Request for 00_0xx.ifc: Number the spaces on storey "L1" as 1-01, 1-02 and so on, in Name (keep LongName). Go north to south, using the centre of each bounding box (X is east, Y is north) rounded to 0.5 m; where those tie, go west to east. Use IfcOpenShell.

First a look at what the model holds.

```python
import ifcopenshell
import ifcopenshell.util.element
import ifcopenshell.util.placement

model = ifcopenshell.open("00_0xx.ifc")
print(model.schema)
storey = next(s for s in model.by_type("IfcBuildingStorey") if s.Name == "L1")
spaces = [e for e in ifcopenshell.util.element.get_decomposition(storey) if e.is_a("IfcSpace")]
for e in sorted(spaces, key=lambda e: e.id()):
    origin = ifcopenshell.util.placement.get_local_placement(e.ObjectPlacement)[:3, 3]
    print(e.id(), e.Name, e.LongName, origin.round(2) + 0.0, sep=" | ")
```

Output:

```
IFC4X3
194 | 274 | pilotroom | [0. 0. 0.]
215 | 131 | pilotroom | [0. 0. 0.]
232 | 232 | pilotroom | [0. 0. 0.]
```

```python
import ifcopenshell
import ifcopenshell.geom
import ifcopenshell.util.element
import ifcopenshell.util.shape

model = ifcopenshell.open("00_0xx.ifc")
settings = ifcopenshell.geom.settings()
settings.set("use-world-coords", True)


def centre(element):
    shape = ifcopenshell.geom.create_shape(settings, element)
    return ifcopenshell.util.shape.get_bbox_centroid(shape.geometry)


storey = next(s for s in model.by_type("IfcBuildingStorey") if s.Name == "L1")
spaces = [e for e in ifcopenshell.util.element.get_decomposition(storey) if e.is_a("IfcSpace")]

# Insertion points can sit at a corner or the storey origin, so sort by the geometry (in metres).
centres = {e: centre(e) for e in spaces}
spaces.sort(key=lambda e: (-round(centres[e][1] / 0.5), centres[e][0]))

for i, e in enumerate(spaces, start=1):
    number = f"1-{i:02d}"
    e.Name = number
    print(e.id(), number)

model.write("00_0xx_v2.ifc")
```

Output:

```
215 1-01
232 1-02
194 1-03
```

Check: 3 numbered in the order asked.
